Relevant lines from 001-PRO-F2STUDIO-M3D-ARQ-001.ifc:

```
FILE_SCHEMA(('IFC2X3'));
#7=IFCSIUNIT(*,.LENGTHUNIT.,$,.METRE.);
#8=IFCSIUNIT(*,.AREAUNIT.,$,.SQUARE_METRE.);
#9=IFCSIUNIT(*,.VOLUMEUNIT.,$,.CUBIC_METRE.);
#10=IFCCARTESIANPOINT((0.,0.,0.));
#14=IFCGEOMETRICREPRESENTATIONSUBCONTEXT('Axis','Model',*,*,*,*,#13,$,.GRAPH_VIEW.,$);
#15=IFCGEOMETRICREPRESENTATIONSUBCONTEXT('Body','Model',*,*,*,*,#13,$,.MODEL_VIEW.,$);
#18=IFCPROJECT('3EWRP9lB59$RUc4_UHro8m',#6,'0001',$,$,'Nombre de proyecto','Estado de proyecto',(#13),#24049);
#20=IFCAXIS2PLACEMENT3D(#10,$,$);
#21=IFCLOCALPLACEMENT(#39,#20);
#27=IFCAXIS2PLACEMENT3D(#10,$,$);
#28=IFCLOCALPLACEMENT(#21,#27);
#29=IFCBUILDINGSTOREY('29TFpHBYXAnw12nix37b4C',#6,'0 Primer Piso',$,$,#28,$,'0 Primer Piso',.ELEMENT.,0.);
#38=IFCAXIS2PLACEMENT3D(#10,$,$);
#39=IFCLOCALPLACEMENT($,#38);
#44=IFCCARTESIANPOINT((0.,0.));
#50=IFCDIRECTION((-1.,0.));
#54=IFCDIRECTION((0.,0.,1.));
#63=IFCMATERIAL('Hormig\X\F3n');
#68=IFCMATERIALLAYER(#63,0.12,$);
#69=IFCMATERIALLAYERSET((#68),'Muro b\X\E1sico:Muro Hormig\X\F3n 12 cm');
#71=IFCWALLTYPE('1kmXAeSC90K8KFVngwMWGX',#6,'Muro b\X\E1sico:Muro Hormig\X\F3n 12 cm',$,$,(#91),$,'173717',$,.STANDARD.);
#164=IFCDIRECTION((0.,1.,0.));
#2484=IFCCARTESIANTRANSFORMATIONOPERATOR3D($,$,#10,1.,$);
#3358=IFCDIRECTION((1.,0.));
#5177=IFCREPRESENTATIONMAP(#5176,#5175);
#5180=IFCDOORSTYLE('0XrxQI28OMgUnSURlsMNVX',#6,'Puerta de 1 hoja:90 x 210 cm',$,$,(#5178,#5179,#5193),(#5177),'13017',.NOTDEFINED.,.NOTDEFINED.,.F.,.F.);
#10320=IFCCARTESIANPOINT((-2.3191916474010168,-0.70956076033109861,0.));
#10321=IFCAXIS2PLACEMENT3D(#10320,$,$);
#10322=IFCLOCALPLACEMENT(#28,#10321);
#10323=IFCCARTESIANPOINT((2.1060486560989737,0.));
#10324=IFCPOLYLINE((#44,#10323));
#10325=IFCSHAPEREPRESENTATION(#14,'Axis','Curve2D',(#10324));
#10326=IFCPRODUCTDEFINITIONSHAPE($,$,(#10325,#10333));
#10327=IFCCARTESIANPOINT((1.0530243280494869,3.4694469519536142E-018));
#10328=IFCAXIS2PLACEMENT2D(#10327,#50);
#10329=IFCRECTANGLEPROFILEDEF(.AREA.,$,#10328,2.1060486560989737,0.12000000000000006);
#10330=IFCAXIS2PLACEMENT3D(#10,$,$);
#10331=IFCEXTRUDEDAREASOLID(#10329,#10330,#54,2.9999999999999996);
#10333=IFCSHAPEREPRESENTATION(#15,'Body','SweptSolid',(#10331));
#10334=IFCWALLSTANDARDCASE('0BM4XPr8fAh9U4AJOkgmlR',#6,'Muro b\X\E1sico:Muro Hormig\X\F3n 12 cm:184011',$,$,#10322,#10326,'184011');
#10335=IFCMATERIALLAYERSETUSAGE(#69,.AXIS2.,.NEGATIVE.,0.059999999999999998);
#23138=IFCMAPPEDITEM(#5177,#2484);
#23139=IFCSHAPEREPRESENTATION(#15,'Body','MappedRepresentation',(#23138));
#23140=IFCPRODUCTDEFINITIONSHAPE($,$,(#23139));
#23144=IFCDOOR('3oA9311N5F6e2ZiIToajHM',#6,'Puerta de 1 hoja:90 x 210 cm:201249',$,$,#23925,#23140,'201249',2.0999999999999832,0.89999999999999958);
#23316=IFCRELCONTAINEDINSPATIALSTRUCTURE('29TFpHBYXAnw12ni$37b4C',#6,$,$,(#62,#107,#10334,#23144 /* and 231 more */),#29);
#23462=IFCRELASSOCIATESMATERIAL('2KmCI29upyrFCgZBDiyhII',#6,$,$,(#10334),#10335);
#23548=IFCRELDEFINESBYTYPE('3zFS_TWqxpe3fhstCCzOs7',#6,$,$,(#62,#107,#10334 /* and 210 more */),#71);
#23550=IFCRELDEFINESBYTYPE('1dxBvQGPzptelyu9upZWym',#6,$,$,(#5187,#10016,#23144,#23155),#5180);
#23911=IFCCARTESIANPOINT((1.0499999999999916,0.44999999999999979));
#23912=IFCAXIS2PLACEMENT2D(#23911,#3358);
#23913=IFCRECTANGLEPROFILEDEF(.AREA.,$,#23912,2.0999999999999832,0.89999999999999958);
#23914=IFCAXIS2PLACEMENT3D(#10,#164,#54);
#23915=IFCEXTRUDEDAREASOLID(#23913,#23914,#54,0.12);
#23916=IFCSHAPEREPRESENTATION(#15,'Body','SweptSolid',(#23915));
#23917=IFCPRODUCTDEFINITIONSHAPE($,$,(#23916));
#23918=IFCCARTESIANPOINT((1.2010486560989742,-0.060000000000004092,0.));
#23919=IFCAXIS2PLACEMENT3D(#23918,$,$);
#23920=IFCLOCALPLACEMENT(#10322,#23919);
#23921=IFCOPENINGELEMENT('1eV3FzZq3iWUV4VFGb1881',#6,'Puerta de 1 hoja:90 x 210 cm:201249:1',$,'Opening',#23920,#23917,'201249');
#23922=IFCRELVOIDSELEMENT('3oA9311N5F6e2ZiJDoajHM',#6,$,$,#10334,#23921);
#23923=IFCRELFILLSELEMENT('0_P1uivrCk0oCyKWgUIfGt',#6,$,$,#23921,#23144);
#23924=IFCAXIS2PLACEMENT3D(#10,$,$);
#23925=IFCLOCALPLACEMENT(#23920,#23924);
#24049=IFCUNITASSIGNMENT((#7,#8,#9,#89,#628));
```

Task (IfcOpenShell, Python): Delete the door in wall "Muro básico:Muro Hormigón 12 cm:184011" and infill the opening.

```python
import ifcopenshell
import ifcopenshell.api.feature
import ifcopenshell.api.root
import ifcopenshell.geom
import ifcopenshell.util.shape

model = ifcopenshell.open("001-PRO-F2STUDIO-M3D-ARQ-001.ifc")
settings = ifcopenshell.geom.settings()


def volume(element):
    """Net volume in cubic metres, openings subtracted."""
    shape = ifcopenshell.geom.create_shape(settings, element)
    return ifcopenshell.util.shape.get_volume(shape.geometry)


door = model.by_guid("3oA9311N5F6e2ZiIToajHM")
opening = door.FillsVoids[0].RelatingOpeningElement
wall = opening.VoidsElements[0].RelatingBuildingElement
before = volume(wall)

ifcopenshell.api.root.remove_product(model, product=door)
ifcopenshell.api.feature.remove_feature(model, feature=opening)

after = volume(wall)

print(f"wall volume {before:.3f} -> {after:.3f} m3")

model.write("001-PRO-F2STUDIO-M3D-ARQ-001_rev.ifc")
```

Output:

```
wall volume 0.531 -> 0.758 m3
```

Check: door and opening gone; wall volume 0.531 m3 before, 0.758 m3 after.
